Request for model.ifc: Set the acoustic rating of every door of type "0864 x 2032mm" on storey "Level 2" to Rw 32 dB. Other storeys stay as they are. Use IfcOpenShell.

First a look at what the model holds.

```python
import ifcopenshell
import ifcopenshell.util.element

model = ifcopenshell.open("model.ifc")
print(model.schema)
storey = next(s for s in model.by_type("IfcBuildingStorey") if s.Name == "Level 2")
doors = [e for e in ifcopenshell.util.element.get_decomposition(storey) if e.is_a("IfcDoor")]
seen = {}
for e in doors:
    element_type = ifcopenshell.util.element.get_type(e)
    key = (element_type.Name if element_type != e and element_type else None, ifcopenshell.util.element.get_pset(e, "Pset_DoorCommon", "AcousticRating"))
    seen[key] = seen.get(key, 0) + 1
for (name, value), count in sorted(seen.items(), key=str):
    print(count, "x", name, "|", value)
```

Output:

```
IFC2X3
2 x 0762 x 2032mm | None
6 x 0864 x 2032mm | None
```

```python
import ifcopenshell
import ifcopenshell.api.pset
import ifcopenshell.util.element

model = ifcopenshell.open("model.ifc")

storey = next(s for s in model.by_type("IfcBuildingStorey") if s.Name == "Level 2")
doors = [e for e in ifcopenshell.util.element.get_decomposition(storey) if e.is_a("IfcDoor")]

count = 0
for e in doors:
    element_type = ifcopenshell.util.element.get_type(e)
    if element_type in (None, e) or element_type.Name != "0864 x 2032mm":
        continue
    # add_pset returns the element's existing set when there is one.
    pset = ifcopenshell.api.pset.add_pset(model, product=e, name="Pset_DoorCommon")
    ifcopenshell.api.pset.edit_pset(model, pset=pset, properties={"AcousticRating": "Rw 32 dB"})
    count += 1

print(count, "doors updated")

model.write("model_updated.ifc")
```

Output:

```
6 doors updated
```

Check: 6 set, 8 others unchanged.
